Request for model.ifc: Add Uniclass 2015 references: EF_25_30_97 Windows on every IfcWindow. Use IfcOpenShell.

First a look at what the model holds.

```python
import ifcopenshell

model = ifcopenshell.open("model.ifc")
print(model.schema)
print("classifications:", [c.Name for c in model.by_type("IfcClassification")])
for ifc_class in ("IfcDoor", "IfcRoof", "IfcStair", "IfcWall", "IfcWindow"):
    print(ifc_class, len(model.by_type(ifc_class)))
```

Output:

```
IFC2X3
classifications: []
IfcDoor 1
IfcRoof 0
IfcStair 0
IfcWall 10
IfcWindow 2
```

```python
import ifcopenshell
import ifcopenshell.api.classification

model = ifcopenshell.open("model.ifc")

# IFC2X3 requires Source and Edition and has no link from the project to the system.
system = model.create_entity("IfcClassification", Source="NBS", Edition="2015", Name="Uniclass 2015")

codes = {
    "IfcWindow": ("EF_25_30_97", "Windows"),
}
for ifc_class, (code, name) in codes.items():
    products = model.by_type(ifc_class)
    ifcopenshell.api.classification.add_reference(
        model, products=products, classification=system, identification=code, name=name
    )
    print(code, len(products))

model.write("model_v2.ifc")
```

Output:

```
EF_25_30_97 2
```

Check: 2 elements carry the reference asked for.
